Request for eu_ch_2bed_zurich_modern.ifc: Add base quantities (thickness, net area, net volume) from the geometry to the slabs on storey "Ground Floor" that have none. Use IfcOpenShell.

First a look at what the model holds.

```python
import ifcopenshell
import ifcopenshell.util.element
import ifcopenshell.util.unit

model = ifcopenshell.open("eu_ch_2bed_zurich_modern.ifc")
print(model.schema)
for unit_type in ("LENGTHUNIT", "AREAUNIT", "VOLUMEUNIT"):
    print(unit_type, ifcopenshell.util.unit.calculate_unit_scale(model, unit_type))
storey = next(s for s in model.by_type("IfcBuildingStorey") if s.Name == "Ground Floor")
slabs = [e for e in ifcopenshell.util.element.get_decomposition(storey) if e.is_a("IfcSlab")]
for e in sorted(slabs, key=lambda e: e.id()):
    print(e.id(), e.is_a(), e.Name, list(ifcopenshell.util.element.get_psets(e, qtos_only=True)), sep=" | ")
```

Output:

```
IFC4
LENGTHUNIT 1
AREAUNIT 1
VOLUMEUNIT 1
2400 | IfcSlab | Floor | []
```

```python
import ifcopenshell
import ifcopenshell.api.pset
import ifcopenshell.geom
import ifcopenshell.util.element
import ifcopenshell.util.shape
import ifcopenshell.util.unit

model = ifcopenshell.open("eu_ch_2bed_zurich_modern.ifc")
unit_scale = ifcopenshell.util.unit.calculate_unit_scale(model)
area_scale = ifcopenshell.util.unit.calculate_unit_scale(model, "AREAUNIT")
volume_scale = ifcopenshell.util.unit.calculate_unit_scale(model, "VOLUMEUNIT")
settings = ifcopenshell.geom.settings()

storey = next(s for s in model.by_type("IfcBuildingStorey") if s.Name == "Ground Floor")
slabs = [e for e in ifcopenshell.util.element.get_decomposition(storey) if e.is_a("IfcSlab")]

for e in sorted(slabs, key=lambda e: e.id()):
    if ifcopenshell.util.element.get_psets(e, qtos_only=True, should_inherit=False):
        continue
    # Geometry comes back in metres, in the element's own axes.
    shape = ifcopenshell.geom.create_shape(settings, e)
    values = {
        "Width": ifcopenshell.util.shape.get_z(shape.geometry) / unit_scale,
        "NetArea": ifcopenshell.util.shape.get_footprint_area(shape.geometry) / area_scale,
        "NetVolume": ifcopenshell.util.shape.get_volume(shape.geometry) / volume_scale,
    }
    qto = ifcopenshell.api.pset.add_qto(model, product=e, name="Qto_SlabBaseQuantities")
    ifcopenshell.api.pset.edit_qto(model, qto=qto, properties=values)
    print(e.id(), {k: round(v, 3) for k, v in values.items()})

model.write("eu_ch_2bed_zurich_modern_rev.ifc")
```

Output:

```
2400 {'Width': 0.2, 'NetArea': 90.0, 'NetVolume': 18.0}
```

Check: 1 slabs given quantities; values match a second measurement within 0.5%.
